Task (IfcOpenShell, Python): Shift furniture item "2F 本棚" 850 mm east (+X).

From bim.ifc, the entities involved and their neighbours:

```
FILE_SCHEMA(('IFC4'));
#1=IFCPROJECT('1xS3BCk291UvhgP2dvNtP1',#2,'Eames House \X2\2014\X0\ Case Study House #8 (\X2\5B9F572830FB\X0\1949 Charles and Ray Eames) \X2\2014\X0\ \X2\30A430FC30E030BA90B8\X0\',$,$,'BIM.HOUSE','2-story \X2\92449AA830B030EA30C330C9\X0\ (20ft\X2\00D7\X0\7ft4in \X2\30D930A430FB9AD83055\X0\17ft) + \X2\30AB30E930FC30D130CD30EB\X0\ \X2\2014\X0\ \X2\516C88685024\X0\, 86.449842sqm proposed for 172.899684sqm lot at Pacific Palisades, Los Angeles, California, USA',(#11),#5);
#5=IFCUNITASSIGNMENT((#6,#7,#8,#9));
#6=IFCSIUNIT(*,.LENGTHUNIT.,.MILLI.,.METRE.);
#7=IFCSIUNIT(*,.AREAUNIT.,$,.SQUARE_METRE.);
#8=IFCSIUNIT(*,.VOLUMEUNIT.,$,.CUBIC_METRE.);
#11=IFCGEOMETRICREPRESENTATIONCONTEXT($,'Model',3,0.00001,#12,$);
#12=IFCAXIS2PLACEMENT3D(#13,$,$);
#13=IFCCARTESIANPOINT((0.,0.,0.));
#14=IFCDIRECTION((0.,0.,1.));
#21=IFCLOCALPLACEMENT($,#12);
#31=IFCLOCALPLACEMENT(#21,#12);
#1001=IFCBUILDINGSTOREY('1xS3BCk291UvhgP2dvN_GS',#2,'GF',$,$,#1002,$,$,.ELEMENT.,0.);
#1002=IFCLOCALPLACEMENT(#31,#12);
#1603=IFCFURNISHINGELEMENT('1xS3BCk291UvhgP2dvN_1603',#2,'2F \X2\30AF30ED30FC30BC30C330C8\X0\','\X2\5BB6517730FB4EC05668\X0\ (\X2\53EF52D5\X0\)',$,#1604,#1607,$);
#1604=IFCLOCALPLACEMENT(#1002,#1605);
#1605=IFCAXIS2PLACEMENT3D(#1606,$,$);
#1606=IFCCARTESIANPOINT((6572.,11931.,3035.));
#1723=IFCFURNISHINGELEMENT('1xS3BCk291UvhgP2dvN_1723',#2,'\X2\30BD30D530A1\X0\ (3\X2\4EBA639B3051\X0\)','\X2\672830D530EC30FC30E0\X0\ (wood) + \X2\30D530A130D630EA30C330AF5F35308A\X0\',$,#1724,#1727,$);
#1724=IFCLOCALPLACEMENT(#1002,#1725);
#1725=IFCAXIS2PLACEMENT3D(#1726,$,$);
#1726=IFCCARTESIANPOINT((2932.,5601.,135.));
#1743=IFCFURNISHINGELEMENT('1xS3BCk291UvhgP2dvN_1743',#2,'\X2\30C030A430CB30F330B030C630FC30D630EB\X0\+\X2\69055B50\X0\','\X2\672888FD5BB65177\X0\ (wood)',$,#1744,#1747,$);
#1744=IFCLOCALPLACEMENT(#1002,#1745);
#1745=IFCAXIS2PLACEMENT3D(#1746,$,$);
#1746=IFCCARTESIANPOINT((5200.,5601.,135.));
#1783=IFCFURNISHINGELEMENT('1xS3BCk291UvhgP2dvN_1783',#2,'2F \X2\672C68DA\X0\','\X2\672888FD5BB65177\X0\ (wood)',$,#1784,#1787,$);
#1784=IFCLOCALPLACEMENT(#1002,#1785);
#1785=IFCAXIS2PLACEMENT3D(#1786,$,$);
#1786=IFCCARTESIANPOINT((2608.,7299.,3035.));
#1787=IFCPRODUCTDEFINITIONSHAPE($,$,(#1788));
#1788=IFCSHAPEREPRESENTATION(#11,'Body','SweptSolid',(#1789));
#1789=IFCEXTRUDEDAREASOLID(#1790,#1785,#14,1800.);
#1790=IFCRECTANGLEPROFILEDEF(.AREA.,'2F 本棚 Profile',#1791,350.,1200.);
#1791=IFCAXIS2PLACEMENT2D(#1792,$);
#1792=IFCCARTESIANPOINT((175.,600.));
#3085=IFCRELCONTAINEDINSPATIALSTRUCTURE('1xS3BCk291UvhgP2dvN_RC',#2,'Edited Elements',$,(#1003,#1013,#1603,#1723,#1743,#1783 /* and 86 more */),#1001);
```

```python
import ifcopenshell
import ifcopenshell.api.geometry
import ifcopenshell.util.placement

model = ifcopenshell.open("bim.ifc")

item = model.by_id(1783)
matrix = ifcopenshell.util.placement.get_local_placement(item.ObjectPlacement)
matrix[0, 3] += 850.0
ifcopenshell.api.geometry.edit_object_placement(model, product=item, matrix=matrix, is_si=False)

print(ifcopenshell.util.placement.get_local_placement(item.ObjectPlacement).round(3) + 0.0)

model.write("bim_rev.ifc")
```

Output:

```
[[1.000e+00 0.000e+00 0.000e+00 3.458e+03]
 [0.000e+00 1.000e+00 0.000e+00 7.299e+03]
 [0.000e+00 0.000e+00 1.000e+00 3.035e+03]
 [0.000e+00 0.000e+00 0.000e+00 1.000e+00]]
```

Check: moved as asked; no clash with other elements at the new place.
